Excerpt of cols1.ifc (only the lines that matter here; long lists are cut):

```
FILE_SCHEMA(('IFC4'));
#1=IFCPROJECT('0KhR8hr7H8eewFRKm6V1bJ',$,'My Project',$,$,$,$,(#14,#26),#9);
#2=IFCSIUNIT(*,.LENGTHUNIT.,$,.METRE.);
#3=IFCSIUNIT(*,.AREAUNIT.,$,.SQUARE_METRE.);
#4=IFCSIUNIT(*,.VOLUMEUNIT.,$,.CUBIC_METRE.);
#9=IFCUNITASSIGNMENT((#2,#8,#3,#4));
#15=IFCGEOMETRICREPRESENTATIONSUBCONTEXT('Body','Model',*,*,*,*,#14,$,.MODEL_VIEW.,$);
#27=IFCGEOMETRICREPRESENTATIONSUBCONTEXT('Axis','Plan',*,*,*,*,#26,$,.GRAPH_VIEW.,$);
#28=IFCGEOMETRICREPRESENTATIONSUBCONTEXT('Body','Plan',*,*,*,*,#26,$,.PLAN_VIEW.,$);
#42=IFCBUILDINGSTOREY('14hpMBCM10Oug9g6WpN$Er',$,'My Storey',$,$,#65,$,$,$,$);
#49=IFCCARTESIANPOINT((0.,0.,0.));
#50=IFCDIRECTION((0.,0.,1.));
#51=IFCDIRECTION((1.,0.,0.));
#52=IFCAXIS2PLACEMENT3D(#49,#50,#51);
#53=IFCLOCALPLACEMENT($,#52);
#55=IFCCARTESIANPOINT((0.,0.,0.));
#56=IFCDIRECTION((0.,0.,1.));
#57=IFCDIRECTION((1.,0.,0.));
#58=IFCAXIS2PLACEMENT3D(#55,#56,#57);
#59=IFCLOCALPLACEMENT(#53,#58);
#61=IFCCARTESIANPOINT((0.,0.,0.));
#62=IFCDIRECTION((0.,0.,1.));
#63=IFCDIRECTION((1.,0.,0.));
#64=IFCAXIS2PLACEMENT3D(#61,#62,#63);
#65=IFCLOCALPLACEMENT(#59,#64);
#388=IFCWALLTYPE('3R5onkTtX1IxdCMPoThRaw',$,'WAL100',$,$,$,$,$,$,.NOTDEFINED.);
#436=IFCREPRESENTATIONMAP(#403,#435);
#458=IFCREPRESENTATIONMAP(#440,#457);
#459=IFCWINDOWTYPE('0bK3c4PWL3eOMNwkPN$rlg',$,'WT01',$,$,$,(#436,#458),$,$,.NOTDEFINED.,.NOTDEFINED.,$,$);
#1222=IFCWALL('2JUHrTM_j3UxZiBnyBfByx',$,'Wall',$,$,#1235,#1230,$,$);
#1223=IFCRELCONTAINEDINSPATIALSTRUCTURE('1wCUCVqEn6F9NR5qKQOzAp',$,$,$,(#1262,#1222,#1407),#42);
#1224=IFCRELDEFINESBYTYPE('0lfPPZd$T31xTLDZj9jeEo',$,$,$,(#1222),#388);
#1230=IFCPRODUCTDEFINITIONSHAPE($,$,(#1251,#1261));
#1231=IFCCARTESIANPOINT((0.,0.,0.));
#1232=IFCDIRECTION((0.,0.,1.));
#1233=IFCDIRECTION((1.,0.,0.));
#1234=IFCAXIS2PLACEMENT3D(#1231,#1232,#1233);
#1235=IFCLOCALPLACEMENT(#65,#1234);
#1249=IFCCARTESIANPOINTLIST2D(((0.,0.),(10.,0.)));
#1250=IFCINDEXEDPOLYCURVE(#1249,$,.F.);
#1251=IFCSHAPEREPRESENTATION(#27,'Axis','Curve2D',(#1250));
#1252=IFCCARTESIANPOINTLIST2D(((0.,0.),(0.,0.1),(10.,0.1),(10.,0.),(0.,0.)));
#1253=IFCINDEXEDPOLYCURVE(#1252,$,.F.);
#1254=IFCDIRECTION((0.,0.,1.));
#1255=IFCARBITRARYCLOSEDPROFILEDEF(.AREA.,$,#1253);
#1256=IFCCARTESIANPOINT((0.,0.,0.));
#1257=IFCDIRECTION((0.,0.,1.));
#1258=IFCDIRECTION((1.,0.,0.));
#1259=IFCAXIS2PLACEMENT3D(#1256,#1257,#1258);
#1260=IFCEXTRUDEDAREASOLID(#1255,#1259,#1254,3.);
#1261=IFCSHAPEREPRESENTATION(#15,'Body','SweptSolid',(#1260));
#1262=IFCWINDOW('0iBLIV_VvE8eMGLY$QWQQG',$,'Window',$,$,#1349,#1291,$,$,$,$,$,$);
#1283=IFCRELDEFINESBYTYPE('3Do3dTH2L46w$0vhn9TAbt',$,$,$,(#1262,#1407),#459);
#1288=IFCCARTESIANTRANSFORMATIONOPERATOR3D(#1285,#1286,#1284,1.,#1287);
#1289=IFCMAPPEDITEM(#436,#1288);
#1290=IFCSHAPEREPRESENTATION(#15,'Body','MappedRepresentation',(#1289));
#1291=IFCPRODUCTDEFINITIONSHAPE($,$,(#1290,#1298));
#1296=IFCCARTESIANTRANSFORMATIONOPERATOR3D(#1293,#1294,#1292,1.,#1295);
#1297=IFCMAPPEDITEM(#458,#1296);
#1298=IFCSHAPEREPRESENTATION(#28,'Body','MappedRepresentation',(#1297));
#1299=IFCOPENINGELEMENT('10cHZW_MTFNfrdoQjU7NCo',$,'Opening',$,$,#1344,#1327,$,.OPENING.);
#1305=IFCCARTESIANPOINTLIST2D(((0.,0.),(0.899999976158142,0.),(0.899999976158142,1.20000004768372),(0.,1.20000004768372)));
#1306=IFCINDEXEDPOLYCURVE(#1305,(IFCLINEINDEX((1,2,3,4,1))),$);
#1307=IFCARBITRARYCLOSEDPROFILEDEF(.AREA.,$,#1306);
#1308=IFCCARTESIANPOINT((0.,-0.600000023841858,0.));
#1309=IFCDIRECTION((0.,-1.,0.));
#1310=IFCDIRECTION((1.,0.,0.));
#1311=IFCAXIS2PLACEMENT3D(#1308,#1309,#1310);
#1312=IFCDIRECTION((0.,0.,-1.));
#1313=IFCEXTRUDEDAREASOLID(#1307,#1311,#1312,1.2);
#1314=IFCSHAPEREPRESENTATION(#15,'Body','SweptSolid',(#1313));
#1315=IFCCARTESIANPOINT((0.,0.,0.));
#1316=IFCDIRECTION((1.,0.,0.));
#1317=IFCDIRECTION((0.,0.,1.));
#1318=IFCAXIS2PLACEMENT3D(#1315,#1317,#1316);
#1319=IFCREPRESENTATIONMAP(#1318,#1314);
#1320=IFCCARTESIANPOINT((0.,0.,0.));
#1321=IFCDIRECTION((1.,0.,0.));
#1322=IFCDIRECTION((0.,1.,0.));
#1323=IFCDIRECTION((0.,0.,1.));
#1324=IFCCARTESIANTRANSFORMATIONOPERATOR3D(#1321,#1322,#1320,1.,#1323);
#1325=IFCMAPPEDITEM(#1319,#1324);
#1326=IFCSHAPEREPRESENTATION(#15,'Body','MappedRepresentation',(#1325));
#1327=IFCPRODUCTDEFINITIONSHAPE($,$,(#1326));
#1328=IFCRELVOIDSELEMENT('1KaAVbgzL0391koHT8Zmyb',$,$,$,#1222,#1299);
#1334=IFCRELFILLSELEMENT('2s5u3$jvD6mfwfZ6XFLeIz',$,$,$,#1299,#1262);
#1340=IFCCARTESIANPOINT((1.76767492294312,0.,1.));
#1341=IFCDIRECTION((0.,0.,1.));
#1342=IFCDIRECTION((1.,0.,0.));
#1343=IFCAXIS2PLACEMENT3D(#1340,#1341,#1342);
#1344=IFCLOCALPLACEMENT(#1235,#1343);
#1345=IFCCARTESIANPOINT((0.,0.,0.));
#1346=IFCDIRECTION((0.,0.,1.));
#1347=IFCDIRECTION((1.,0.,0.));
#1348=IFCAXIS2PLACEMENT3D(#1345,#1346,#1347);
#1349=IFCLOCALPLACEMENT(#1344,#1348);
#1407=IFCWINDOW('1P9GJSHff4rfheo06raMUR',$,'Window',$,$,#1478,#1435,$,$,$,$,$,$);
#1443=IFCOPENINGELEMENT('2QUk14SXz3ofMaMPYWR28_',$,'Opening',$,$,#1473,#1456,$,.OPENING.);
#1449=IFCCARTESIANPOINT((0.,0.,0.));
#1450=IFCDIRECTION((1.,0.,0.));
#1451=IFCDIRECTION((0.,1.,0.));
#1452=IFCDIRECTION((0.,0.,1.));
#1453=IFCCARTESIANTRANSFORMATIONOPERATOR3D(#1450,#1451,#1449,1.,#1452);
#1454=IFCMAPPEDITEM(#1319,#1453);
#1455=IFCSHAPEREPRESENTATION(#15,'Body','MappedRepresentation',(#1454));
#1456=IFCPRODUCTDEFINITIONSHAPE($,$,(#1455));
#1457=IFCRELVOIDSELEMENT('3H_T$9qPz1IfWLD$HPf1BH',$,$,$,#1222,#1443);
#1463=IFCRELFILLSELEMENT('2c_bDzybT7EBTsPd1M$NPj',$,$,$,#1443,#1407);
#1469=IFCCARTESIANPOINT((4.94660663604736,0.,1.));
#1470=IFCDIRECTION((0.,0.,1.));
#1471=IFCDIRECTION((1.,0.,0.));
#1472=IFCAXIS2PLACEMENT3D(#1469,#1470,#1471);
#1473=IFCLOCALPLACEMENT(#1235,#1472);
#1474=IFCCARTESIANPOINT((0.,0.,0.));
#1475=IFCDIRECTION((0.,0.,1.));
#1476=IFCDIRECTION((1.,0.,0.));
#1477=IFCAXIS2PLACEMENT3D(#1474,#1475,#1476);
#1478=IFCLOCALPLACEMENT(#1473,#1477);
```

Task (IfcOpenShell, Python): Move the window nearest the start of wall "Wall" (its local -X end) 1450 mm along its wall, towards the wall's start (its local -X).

```python
import ifcopenshell
import ifcopenshell.api.geometry
import ifcopenshell.util.placement

model = ifcopenshell.open("cols1.ifc")

window = model.by_guid("0iBLIV_VvE8eMGLY$QWQQG")
opening = window.FillsVoids[0].RelatingOpeningElement
wall = opening.VoidsElements[0].RelatingBuildingElement

wall_matrix = ifcopenshell.util.placement.get_local_placement(wall.ObjectPlacement)
shift = wall_matrix[:3, 0] * -1.45
before = ifcopenshell.util.placement.get_local_placement(window.ObjectPlacement)[:3, 3].copy()

# The window is placed relative to its opening, so it follows when the opening moves.
matrix = ifcopenshell.util.placement.get_local_placement(opening.ObjectPlacement)
matrix[:3, 3] += shift
ifcopenshell.api.geometry.edit_object_placement(
    model, product=opening, matrix=matrix, is_si=False, should_transform_children=True
)

after = ifcopenshell.util.placement.get_local_placement(window.ObjectPlacement)[:3, 3]
print("window moved by", (after - before).round(3) + 0.0)

model.write("cols1-out.ifc")
```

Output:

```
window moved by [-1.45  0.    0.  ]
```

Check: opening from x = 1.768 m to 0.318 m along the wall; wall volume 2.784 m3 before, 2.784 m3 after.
